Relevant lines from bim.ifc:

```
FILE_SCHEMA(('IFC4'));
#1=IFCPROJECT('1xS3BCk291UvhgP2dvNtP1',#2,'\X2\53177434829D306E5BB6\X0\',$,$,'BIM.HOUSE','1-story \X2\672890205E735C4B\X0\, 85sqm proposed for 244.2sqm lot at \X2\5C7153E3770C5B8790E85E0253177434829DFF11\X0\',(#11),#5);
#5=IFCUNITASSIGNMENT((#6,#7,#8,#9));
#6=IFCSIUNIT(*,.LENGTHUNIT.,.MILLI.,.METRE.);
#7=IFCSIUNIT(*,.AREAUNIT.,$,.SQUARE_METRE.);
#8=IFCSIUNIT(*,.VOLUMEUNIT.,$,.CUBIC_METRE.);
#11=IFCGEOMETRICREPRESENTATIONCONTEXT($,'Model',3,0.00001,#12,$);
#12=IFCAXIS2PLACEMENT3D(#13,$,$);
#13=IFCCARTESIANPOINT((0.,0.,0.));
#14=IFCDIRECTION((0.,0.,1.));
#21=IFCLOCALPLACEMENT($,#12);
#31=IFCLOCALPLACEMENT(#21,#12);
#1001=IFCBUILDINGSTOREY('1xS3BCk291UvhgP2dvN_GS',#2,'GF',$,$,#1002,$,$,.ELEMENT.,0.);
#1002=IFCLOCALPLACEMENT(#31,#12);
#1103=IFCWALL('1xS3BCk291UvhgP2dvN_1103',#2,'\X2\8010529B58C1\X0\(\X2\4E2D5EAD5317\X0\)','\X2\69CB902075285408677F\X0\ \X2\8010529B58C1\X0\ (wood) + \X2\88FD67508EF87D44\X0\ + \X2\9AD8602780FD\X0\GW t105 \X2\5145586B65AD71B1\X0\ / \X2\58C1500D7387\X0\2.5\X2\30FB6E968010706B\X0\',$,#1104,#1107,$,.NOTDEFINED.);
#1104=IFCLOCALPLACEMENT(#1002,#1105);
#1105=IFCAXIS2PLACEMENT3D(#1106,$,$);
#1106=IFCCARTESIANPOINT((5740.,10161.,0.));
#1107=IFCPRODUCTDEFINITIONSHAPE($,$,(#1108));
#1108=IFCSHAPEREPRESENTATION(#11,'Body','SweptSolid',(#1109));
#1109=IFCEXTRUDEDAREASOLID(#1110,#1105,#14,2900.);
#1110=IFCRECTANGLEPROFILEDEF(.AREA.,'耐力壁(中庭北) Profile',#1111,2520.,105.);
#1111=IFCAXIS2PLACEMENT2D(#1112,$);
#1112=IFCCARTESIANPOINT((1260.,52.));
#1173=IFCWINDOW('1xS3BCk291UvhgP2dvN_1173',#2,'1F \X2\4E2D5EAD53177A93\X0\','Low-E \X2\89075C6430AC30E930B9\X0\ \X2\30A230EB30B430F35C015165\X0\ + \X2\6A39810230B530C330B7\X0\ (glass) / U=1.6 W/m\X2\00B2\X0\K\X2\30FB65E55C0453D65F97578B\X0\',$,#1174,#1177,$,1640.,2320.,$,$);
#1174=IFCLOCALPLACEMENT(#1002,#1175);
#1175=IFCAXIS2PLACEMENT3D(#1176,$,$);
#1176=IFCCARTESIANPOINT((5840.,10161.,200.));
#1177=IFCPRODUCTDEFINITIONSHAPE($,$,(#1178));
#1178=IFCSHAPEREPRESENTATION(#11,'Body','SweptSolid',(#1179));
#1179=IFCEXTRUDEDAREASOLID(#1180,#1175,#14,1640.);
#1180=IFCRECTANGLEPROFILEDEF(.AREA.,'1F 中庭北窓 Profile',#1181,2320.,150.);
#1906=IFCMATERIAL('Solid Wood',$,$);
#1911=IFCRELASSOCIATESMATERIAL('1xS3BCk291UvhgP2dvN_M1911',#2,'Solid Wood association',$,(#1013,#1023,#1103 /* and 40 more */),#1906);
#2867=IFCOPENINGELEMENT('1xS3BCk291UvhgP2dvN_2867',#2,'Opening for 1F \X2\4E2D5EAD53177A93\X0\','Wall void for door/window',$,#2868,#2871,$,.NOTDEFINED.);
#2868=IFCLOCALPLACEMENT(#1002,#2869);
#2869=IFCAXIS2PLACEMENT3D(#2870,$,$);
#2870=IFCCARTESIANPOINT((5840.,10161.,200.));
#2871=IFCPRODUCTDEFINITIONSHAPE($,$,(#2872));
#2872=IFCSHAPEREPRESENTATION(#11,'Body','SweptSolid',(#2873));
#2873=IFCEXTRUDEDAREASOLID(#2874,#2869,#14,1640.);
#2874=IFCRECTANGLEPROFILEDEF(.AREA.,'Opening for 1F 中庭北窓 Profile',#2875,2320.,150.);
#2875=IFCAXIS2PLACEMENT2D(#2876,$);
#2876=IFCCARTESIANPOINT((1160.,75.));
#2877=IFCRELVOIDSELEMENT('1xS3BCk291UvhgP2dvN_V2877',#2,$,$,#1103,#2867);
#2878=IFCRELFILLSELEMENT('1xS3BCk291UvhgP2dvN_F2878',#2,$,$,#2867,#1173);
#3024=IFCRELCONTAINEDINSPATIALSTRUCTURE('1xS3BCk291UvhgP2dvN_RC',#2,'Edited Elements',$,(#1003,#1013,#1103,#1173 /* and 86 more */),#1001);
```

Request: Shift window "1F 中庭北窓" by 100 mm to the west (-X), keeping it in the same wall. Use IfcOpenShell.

```python
import ifcopenshell
import ifcopenshell.api.geometry
import ifcopenshell.util.placement
import ifcopenshell.util.unit

model = ifcopenshell.open("bim.ifc")
unit_scale = ifcopenshell.util.unit.calculate_unit_scale(model)

window = model.by_guid("1xS3BCk291UvhgP2dvN_1173")
opening = window.FillsVoids[0].RelatingOpeningElement
wall = opening.VoidsElements[0].RelatingBuildingElement

wall_matrix = ifcopenshell.util.placement.get_local_placement(wall.ObjectPlacement)
shift = wall_matrix[:3, 0] * -0.1 / unit_scale
before = ifcopenshell.util.placement.get_local_placement(window.ObjectPlacement)[:3, 3].copy()

# The window is not placed relative to its opening, so move both.
for product in (opening, window):
    matrix = ifcopenshell.util.placement.get_local_placement(product.ObjectPlacement)
    matrix[:3, 3] += shift
    ifcopenshell.api.geometry.edit_object_placement(model, product=product, matrix=matrix, is_si=False)

after = ifcopenshell.util.placement.get_local_placement(window.ObjectPlacement)[:3, 3]
print("window moved by", (after - before).round(3) + 0.0)

model.write("bim-out.ifc")
```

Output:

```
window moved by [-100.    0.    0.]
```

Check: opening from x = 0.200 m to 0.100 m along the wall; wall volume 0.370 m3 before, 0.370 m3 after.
